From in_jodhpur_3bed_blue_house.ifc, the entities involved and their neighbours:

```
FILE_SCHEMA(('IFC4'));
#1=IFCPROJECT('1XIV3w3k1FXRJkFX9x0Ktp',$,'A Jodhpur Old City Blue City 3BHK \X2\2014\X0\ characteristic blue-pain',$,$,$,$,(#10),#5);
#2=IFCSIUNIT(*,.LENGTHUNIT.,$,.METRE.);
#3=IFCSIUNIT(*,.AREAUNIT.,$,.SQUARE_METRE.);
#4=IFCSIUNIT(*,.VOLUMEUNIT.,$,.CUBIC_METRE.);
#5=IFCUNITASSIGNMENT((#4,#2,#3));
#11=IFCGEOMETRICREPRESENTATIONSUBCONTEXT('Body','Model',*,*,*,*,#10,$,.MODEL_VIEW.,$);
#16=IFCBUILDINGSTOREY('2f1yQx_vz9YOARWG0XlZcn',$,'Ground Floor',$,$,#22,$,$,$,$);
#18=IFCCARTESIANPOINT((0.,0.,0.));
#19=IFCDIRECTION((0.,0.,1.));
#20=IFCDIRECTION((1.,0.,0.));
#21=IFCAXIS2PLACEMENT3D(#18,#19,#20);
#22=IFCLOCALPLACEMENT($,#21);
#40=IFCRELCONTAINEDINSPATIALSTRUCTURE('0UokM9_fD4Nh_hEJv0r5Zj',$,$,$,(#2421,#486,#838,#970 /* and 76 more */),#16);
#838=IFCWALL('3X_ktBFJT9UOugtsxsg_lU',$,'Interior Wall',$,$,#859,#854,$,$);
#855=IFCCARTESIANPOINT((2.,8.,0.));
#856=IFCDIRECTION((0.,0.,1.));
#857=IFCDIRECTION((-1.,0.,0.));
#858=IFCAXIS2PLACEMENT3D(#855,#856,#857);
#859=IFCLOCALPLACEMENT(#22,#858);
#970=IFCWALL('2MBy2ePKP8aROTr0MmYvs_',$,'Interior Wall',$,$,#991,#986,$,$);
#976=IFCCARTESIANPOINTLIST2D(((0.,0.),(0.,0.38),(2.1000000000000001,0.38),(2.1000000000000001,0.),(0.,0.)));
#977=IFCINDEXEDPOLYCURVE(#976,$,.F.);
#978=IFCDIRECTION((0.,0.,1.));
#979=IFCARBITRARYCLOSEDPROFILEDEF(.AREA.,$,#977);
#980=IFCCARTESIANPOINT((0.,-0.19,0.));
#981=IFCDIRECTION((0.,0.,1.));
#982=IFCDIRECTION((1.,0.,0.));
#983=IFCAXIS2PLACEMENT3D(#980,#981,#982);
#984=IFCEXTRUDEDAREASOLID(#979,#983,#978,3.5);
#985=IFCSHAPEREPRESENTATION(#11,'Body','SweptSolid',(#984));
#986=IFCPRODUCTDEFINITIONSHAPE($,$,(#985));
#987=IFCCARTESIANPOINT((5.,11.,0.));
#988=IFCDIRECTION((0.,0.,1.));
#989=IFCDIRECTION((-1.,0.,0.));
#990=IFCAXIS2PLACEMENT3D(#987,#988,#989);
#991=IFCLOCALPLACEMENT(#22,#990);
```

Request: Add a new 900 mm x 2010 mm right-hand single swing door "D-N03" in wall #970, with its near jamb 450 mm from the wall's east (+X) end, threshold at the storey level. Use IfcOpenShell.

```python
import numpy as np
import ifcopenshell
import ifcopenshell.api.feature
import ifcopenshell.api.geometry
import ifcopenshell.api.root
import ifcopenshell.api.spatial
import ifcopenshell.geom
import ifcopenshell.util.element
import ifcopenshell.util.placement
import ifcopenshell.util.representation
import ifcopenshell.util.shape
import ifcopenshell.util.unit

model = ifcopenshell.open("in_jodhpur_3bed_blue_house.ifc")
unit_scale = ifcopenshell.util.unit.calculate_unit_scale(model)
settings = ifcopenshell.geom.settings()


def volume(element):
    """Net volume in cubic metres, openings subtracted."""
    shape = ifcopenshell.geom.create_shape(settings, element)
    return ifcopenshell.util.shape.get_volume(shape.geometry)


wall = model.by_guid("2MBy2ePKP8aROTr0MmYvs_")
storey = ifcopenshell.util.element.get_container(wall, ifc_class="IfcBuildingStorey")
context = ifcopenshell.util.representation.get_context(model, "Model", "Body", "MODEL_VIEW")
before = volume(wall)

width, height, from_end, sill = 0.9, 2.01, 0.45, 0.0  # metres

# The wall runs along its own X axis, and the end named is its -X end.
wall_shape = ifcopenshell.geom.create_shape(settings, wall)
x, y, z = ifcopenshell.util.shape.get_vertices(wall_shape.geometry).T
start = x.min() + from_end
face, thickness = float(y.min()), float(y.max() - y.min())
wall_matrix = ifcopenshell.util.placement.get_local_placement(wall.ObjectPlacement)
level = ifcopenshell.util.placement.get_local_placement(storey.ObjectPlacement)[2, 3]


def in_wall(x, y):
    """Placement at x, y metres in the wall's axes, at sill height."""
    matrix = wall_matrix.copy()
    matrix[:, 3] = wall_matrix @ np.array([x / unit_scale, y / unit_scale, 0.0, 1.0])
    matrix[2, 3] = level + sill / unit_scale
    return matrix


# Opening: a box that overshoots both wall faces by 50 mm.
opening = ifcopenshell.api.root.create_entity(model, ifc_class="IfcOpeningElement", predefined_type="OPENING")
box = ifcopenshell.api.geometry.add_wall_representation(
    model, context=context, length=width, height=height, thickness=thickness + 0.1
)
ifcopenshell.api.geometry.assign_representation(model, product=opening, representation=box)
ifcopenshell.api.geometry.edit_object_placement(model, product=opening, matrix=in_wall(start, face - 0.05), is_si=False)
ifcopenshell.api.feature.add_feature(model, feature=opening, element=wall)

door = ifcopenshell.api.root.create_entity(model, ifc_class="IfcDoor", name="D-N03", predefined_type="DOOR")
door.OverallWidth, door.OverallHeight = width / unit_scale, height / unit_scale
door.OperationType = "SINGLE_SWING_RIGHT"
body = ifcopenshell.api.geometry.add_door_representation(
    model,
    context=context,
    overall_width=door.OverallWidth,
    overall_height=door.OverallHeight,
    operation_type="SINGLE_SWING_RIGHT",
    lining_properties={"LiningDepth": thickness / unit_scale, "ThresholdDepth": thickness / unit_scale},
)
ifcopenshell.api.geometry.assign_representation(model, product=door, representation=body)
ifcopenshell.api.spatial.assign_container(model, products=[door], relating_structure=storey)
ifcopenshell.api.feature.add_filling(model, opening=opening, element=door)

# The lining spans the wall, so the door starts at the wall face.
ifcopenshell.api.geometry.edit_object_placement(model, product=door, matrix=in_wall(start, face), is_si=False)

after = volume(wall)

print(f"wall volume {before:.3f} -> {after:.3f} m3")

model.write("in_jodhpur_3bed_blue_house_edited.ifc")
```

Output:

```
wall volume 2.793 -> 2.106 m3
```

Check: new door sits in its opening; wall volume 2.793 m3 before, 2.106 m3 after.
